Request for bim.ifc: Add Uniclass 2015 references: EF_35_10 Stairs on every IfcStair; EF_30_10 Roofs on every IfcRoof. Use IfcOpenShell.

First a look at what the model holds.

```python
import ifcopenshell

model = ifcopenshell.open("bim.ifc")
print(model.schema)
print("classifications:", [c.Name for c in model.by_type("IfcClassification")])
for ifc_class in ("IfcDoor", "IfcRoof", "IfcStair", "IfcWall", "IfcWindow"):
    print(ifc_class, len(model.by_type(ifc_class)))
```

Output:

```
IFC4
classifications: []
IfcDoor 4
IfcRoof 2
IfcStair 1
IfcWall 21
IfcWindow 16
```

```python
import ifcopenshell
import ifcopenshell.api.classification

model = ifcopenshell.open("bim.ifc")

system = ifcopenshell.api.classification.add_classification(model, classification="Uniclass 2015")

codes = {
    "IfcStair": ("EF_35_10", "Stairs"),
    "IfcRoof": ("EF_30_10", "Roofs"),
}
for ifc_class, (code, name) in codes.items():
    products = model.by_type(ifc_class)
    ifcopenshell.api.classification.add_reference(
        model, products=products, classification=system, identification=code, name=name
    )
    print(code, len(products))

model.write("bim_rev.ifc")
```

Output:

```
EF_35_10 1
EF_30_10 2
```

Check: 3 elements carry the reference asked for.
